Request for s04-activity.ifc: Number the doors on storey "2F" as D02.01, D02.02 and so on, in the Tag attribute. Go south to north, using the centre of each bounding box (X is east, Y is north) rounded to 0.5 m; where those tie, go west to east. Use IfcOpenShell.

First a look at what the model holds.

```python
import ifcopenshell
import ifcopenshell.util.element
import ifcopenshell.util.placement

model = ifcopenshell.open("s04-activity.ifc")
print(model.schema)
storey = next(s for s in model.by_type("IfcBuildingStorey") if s.Name == "2F")
doors = [e for e in ifcopenshell.util.element.get_decomposition(storey) if e.is_a("IfcDoor")]
for e in sorted(doors, key=lambda e: e.id()):
    origin = ifcopenshell.util.placement.get_local_placement(e.ObjectPlacement)[:3, 3]
    print(e.id(), e.Tag, e.Name, origin.round(2) + 0.0, sep=" | ")
```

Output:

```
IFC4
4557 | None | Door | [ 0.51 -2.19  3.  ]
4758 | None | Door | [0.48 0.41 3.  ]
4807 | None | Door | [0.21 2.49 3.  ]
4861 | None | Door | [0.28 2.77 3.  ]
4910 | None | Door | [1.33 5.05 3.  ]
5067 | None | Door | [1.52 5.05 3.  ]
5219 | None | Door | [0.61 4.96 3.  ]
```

```python
import ifcopenshell
import ifcopenshell.geom
import ifcopenshell.util.element
import ifcopenshell.util.shape

model = ifcopenshell.open("s04-activity.ifc")
settings = ifcopenshell.geom.settings()
settings.set("use-world-coords", True)


def centre(element):
    shape = ifcopenshell.geom.create_shape(settings, element)
    return ifcopenshell.util.shape.get_bbox_centroid(shape.geometry)


storey = next(s for s in model.by_type("IfcBuildingStorey") if s.Name == "2F")
doors = [e for e in ifcopenshell.util.element.get_decomposition(storey) if e.is_a("IfcDoor")]

# Insertion points can sit at a corner or the storey origin, so sort by the geometry (in metres).
centres = {e: centre(e) for e in doors}
doors.sort(key=lambda e: (round(centres[e][1] / 0.5), centres[e][0]))

for i, e in enumerate(doors, start=1):
    number = f"D02.{i:02d}"
    e.Tag = number
    print(e.id(), number)

model.write("s04-activity-out.ifc")
```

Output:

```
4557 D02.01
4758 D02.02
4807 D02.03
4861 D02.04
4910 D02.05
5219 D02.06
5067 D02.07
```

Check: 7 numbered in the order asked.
